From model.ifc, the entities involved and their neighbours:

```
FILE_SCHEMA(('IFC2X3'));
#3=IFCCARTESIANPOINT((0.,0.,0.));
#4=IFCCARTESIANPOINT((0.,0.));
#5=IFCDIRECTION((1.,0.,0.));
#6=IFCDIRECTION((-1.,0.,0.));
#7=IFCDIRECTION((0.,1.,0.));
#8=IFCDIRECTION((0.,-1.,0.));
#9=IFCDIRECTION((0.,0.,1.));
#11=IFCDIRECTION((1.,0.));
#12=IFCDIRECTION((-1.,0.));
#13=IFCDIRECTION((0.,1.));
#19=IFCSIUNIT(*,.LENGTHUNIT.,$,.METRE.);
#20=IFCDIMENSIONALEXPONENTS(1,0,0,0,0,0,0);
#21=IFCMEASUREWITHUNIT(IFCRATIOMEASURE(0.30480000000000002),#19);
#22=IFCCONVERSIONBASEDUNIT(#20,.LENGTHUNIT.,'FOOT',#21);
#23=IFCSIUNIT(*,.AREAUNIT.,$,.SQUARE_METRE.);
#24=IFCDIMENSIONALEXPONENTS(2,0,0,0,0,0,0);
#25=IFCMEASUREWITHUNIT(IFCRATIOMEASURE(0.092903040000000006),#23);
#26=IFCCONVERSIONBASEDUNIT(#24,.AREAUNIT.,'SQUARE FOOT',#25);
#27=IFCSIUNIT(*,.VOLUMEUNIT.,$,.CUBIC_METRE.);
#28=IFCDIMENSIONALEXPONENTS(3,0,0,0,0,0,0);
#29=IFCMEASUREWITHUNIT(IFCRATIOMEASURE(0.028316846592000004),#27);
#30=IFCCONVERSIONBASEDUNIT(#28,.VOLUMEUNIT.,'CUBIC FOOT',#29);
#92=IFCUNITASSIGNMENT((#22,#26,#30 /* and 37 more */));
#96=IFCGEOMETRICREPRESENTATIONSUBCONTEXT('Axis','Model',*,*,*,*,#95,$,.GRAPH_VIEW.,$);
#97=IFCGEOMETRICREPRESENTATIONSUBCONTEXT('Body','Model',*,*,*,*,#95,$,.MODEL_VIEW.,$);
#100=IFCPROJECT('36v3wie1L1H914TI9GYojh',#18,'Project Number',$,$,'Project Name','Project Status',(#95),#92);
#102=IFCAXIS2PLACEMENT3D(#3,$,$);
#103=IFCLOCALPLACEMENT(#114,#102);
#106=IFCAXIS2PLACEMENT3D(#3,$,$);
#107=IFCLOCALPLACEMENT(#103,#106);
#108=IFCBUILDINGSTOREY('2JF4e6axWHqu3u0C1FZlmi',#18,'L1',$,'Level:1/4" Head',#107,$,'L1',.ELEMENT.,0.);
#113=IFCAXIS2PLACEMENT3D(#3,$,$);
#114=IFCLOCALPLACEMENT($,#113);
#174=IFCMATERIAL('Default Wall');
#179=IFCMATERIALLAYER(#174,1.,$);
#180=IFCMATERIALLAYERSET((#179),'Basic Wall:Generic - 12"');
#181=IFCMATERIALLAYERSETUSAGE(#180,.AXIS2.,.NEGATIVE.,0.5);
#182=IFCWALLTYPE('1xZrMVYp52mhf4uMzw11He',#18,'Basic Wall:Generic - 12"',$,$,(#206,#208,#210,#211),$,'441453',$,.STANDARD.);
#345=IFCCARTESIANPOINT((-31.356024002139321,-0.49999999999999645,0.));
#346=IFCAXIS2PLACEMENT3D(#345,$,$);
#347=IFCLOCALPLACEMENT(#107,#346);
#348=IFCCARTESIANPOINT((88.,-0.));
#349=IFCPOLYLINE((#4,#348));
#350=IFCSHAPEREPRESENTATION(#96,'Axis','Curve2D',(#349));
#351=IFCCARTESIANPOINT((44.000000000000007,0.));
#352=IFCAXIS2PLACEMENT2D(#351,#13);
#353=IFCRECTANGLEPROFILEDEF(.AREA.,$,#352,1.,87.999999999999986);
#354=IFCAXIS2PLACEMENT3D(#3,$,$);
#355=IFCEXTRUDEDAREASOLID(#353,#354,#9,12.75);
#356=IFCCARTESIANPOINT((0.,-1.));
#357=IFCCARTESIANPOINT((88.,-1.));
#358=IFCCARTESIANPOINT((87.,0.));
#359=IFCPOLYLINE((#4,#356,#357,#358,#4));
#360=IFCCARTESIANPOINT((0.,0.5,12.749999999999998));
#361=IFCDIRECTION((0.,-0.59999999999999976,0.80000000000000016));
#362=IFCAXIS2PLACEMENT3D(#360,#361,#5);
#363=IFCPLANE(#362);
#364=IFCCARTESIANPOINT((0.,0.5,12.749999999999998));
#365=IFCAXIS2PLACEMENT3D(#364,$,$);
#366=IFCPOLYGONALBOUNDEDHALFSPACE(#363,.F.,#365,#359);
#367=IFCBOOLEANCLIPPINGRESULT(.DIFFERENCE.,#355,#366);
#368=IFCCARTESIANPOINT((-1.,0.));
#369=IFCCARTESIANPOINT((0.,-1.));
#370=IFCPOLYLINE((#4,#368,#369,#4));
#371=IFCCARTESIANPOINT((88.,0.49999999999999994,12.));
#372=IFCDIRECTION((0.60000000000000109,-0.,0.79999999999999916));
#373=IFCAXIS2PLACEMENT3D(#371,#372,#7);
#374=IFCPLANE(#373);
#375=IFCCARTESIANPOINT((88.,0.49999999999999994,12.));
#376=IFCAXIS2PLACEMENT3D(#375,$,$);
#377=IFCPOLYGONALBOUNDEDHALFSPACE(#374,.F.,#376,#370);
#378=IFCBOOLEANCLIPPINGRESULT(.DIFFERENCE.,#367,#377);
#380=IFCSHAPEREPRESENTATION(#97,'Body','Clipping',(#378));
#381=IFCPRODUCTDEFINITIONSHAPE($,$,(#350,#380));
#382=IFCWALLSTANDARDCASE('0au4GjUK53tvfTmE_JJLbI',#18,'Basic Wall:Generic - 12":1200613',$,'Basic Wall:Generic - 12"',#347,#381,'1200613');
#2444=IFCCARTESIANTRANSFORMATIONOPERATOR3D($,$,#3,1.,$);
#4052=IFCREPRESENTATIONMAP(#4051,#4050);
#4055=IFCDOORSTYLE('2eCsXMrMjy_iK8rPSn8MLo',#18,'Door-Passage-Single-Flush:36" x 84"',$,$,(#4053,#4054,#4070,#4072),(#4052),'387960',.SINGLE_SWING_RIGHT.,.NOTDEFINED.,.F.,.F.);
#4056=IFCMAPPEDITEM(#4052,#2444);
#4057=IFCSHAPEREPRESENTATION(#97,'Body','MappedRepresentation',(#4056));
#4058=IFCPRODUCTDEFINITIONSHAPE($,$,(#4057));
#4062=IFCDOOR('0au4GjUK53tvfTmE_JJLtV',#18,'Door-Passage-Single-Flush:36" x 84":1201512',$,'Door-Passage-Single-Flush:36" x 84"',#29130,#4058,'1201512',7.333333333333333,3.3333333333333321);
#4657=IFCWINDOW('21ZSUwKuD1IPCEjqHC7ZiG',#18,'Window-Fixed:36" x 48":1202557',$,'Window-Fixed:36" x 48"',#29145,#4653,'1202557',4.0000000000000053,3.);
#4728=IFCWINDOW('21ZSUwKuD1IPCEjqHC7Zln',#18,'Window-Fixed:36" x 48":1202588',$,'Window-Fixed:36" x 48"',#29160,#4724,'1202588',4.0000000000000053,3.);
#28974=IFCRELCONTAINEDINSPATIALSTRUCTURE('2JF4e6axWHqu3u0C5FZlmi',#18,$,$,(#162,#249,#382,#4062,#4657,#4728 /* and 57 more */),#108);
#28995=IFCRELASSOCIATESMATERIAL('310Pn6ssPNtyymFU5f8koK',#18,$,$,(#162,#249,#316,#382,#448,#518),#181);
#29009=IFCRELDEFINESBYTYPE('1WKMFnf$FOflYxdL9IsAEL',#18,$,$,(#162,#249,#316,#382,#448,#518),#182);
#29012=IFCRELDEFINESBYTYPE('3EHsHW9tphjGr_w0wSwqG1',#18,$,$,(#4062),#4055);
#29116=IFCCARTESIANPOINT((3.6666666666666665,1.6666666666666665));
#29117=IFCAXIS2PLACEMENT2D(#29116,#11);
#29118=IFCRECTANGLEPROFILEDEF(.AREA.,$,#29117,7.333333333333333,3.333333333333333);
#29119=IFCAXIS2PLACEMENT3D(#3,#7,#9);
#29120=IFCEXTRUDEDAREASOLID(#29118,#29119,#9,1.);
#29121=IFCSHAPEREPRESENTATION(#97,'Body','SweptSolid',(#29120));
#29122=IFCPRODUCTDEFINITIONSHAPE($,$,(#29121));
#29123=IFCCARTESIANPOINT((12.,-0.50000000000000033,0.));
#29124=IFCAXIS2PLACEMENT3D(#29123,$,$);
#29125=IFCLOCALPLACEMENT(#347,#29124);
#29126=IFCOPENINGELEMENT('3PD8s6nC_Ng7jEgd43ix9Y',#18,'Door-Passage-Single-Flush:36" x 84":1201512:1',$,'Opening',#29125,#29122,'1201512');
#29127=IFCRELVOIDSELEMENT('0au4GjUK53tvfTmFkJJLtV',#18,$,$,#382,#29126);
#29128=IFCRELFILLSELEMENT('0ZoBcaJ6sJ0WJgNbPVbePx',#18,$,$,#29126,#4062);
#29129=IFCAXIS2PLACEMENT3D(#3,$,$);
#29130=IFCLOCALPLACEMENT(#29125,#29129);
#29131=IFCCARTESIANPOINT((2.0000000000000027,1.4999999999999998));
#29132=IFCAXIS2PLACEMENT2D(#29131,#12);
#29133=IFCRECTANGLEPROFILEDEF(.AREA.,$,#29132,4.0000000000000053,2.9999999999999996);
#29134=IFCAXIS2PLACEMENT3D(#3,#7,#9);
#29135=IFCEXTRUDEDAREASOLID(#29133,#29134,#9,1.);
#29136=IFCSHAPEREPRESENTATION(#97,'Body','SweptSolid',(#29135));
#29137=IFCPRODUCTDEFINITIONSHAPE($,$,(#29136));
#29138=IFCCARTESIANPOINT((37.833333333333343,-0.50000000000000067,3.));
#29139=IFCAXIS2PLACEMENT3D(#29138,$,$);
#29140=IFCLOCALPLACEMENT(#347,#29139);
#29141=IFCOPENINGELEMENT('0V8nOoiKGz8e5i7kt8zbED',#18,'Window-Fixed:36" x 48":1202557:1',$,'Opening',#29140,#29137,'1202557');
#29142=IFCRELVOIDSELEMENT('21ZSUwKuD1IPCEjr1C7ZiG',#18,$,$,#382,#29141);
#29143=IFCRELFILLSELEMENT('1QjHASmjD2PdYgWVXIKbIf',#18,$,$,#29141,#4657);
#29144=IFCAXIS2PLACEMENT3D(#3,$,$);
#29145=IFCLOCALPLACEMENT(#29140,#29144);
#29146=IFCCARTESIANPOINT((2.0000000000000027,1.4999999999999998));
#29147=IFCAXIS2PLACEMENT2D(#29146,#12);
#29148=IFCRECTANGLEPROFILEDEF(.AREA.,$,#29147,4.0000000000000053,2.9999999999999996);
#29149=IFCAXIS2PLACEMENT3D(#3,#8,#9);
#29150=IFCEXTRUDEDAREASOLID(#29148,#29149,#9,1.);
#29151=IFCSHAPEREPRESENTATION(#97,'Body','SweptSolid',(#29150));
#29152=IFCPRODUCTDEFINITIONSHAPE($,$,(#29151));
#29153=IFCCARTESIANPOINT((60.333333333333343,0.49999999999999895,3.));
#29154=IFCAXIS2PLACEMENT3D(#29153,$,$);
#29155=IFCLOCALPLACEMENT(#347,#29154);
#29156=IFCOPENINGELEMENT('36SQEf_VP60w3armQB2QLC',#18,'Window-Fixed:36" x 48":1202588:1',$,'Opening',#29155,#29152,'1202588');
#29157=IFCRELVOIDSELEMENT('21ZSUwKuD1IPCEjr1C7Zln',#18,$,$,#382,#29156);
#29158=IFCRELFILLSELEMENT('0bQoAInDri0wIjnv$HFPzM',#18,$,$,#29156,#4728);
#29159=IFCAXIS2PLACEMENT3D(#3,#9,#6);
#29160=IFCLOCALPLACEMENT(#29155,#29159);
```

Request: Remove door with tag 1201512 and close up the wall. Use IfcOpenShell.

```python
import ifcopenshell
import ifcopenshell.api.feature
import ifcopenshell.api.root
import ifcopenshell.geom
import ifcopenshell.util.shape

model = ifcopenshell.open("model.ifc")
settings = ifcopenshell.geom.settings()


def volume(element):
    """Net volume in cubic metres, openings subtracted."""
    shape = ifcopenshell.geom.create_shape(settings, element)
    return ifcopenshell.util.shape.get_volume(shape.geometry)


door = model.by_guid("0au4GjUK53tvfTmE_JJLtV")
opening = door.FillsVoids[0].RelatingOpeningElement
wall = opening.VoidsElements[0].RelatingBuildingElement
before = volume(wall)

ifcopenshell.api.root.remove_product(model, product=door)
ifcopenshell.api.feature.remove_feature(model, feature=opening)

after = volume(wall)

print(f"wall volume {before:.3f} -> {after:.3f} m3")

model.write("model_v2.ifc")
```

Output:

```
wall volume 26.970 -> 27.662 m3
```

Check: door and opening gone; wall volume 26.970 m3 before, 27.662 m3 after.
